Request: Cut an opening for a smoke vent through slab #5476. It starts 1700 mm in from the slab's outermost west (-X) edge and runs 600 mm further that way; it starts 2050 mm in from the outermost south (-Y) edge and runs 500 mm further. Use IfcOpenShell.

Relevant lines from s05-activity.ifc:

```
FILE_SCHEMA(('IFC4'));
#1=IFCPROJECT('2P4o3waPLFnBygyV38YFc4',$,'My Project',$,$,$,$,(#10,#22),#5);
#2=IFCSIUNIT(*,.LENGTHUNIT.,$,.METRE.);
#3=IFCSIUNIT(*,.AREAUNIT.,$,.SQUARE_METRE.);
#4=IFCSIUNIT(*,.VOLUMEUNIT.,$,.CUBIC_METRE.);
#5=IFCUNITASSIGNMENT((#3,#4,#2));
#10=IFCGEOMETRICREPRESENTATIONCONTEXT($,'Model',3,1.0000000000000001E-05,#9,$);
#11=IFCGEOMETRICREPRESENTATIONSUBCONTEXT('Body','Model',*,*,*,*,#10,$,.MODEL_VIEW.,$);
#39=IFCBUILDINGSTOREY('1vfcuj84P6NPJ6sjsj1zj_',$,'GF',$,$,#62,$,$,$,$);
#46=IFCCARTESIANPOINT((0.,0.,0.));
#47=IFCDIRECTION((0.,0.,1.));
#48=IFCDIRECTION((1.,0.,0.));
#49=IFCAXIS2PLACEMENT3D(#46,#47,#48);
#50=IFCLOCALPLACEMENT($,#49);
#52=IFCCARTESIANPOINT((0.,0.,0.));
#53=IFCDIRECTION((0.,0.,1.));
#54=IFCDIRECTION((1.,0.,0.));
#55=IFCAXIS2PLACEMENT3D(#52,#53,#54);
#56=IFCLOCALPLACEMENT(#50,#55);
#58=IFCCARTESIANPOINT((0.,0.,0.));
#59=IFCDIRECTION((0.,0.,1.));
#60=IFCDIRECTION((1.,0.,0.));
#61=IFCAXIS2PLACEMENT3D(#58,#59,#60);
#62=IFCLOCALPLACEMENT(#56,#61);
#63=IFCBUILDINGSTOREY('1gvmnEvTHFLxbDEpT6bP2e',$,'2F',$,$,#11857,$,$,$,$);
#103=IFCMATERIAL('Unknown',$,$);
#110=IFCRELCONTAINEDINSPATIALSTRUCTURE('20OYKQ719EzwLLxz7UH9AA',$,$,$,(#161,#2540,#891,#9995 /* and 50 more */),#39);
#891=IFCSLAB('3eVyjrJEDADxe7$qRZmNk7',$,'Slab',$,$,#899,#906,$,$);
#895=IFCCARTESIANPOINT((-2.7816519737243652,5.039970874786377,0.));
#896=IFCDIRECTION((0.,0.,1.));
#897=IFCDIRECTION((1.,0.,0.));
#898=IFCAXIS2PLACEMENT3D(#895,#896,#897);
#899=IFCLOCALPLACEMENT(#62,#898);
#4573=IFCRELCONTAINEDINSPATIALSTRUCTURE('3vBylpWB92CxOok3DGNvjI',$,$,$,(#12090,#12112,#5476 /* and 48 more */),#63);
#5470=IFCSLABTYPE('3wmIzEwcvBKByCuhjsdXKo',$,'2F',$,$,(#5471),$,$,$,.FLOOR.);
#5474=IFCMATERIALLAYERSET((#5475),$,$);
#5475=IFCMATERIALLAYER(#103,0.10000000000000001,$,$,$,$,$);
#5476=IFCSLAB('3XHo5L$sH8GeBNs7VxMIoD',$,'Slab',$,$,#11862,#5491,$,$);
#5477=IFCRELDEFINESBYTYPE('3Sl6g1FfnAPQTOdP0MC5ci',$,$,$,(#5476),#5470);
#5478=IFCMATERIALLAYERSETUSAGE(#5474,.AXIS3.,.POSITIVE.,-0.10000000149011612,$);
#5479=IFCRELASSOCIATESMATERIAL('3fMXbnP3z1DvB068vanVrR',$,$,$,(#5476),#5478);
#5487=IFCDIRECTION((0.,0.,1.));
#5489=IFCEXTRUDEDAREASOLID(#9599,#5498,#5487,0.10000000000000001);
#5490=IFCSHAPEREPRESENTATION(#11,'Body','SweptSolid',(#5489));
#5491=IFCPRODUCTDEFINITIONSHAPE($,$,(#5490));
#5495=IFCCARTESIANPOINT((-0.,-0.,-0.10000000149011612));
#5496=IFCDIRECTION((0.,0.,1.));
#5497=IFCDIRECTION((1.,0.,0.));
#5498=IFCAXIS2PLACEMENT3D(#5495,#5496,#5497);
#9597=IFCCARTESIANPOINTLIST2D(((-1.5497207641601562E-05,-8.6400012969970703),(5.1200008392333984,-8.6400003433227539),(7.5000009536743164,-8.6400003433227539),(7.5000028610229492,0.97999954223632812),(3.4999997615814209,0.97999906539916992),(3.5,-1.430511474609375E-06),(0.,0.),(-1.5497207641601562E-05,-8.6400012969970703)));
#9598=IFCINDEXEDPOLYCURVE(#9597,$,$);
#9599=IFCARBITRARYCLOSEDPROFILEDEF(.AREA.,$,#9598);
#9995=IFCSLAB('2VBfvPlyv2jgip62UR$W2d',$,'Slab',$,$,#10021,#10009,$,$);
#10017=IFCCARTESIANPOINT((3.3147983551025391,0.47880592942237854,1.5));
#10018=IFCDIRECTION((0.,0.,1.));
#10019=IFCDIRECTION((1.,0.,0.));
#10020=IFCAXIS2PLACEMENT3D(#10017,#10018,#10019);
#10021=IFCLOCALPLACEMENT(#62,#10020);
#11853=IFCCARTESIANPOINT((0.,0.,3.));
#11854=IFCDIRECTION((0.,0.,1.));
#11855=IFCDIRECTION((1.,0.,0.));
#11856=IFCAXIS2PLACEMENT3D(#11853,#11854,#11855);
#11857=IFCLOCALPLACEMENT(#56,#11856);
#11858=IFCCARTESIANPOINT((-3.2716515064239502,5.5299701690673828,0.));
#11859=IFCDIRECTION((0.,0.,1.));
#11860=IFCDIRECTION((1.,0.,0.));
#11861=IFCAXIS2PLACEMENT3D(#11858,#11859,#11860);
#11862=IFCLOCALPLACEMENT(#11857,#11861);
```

```python
import numpy as np
import ifcopenshell
import ifcopenshell.api.feature
import ifcopenshell.api.geometry
import ifcopenshell.api.root
import ifcopenshell.geom
import ifcopenshell.util.placement
import ifcopenshell.util.representation
import ifcopenshell.util.shape
import ifcopenshell.util.unit

model = ifcopenshell.open("s05-activity.ifc")
unit_scale = ifcopenshell.util.unit.calculate_unit_scale(model)
settings = ifcopenshell.geom.settings()


def volume(element):
    """Net volume in cubic metres, openings subtracted."""
    shape = ifcopenshell.geom.create_shape(settings, element)
    return ifcopenshell.util.shape.get_volume(shape.geometry)


slab = model.by_id(5476)
before = volume(slab)

# Extent in the slab's own axes, in metres. The edges named are its -X and -Y sides.
slab_shape = ifcopenshell.geom.create_shape(settings, slab)
vertices = ifcopenshell.util.shape.get_vertices(slab_shape.geometry)
x_min, y_min, bottom = vertices.min(axis=0)
top = vertices[:, 2].max()

opening = ifcopenshell.api.root.create_entity(model, ifc_class="IfcOpeningElement", name="Smoke vent opening", predefined_type="OPENING")
context = ifcopenshell.util.representation.get_context(model, "Model", "Body", "MODEL_VIEW")
width, depth = 0.6, 0.5
outline = [(0.0, 0.0), (width, 0.0), (width, depth), (0.0, depth), (0.0, 0.0)]
# Overshoot both faces by 50 mm so the cut is clean.
shape = ifcopenshell.api.geometry.add_slab_representation(
    model, context=context, depth=top - bottom + 0.1, polyline=outline
)
ifcopenshell.api.geometry.assign_representation(model, product=opening, representation=shape)

matrix = ifcopenshell.util.placement.get_local_placement(slab.ObjectPlacement)
matrix[:, 3] = matrix @ np.append(np.array([x_min + 1.7, y_min + 2.05, bottom - 0.05]) / unit_scale, 1.0)
ifcopenshell.api.geometry.edit_object_placement(model, product=opening, matrix=matrix, is_si=False)
ifcopenshell.api.feature.add_feature(model, feature=opening, element=slab)

after = volume(slab)

print(f"slab volume {before:.3f} -> {after:.3f} m3")

model.write("s05-activity-out.ifc")
```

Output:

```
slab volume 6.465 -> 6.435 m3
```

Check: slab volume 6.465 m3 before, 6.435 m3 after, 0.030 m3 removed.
